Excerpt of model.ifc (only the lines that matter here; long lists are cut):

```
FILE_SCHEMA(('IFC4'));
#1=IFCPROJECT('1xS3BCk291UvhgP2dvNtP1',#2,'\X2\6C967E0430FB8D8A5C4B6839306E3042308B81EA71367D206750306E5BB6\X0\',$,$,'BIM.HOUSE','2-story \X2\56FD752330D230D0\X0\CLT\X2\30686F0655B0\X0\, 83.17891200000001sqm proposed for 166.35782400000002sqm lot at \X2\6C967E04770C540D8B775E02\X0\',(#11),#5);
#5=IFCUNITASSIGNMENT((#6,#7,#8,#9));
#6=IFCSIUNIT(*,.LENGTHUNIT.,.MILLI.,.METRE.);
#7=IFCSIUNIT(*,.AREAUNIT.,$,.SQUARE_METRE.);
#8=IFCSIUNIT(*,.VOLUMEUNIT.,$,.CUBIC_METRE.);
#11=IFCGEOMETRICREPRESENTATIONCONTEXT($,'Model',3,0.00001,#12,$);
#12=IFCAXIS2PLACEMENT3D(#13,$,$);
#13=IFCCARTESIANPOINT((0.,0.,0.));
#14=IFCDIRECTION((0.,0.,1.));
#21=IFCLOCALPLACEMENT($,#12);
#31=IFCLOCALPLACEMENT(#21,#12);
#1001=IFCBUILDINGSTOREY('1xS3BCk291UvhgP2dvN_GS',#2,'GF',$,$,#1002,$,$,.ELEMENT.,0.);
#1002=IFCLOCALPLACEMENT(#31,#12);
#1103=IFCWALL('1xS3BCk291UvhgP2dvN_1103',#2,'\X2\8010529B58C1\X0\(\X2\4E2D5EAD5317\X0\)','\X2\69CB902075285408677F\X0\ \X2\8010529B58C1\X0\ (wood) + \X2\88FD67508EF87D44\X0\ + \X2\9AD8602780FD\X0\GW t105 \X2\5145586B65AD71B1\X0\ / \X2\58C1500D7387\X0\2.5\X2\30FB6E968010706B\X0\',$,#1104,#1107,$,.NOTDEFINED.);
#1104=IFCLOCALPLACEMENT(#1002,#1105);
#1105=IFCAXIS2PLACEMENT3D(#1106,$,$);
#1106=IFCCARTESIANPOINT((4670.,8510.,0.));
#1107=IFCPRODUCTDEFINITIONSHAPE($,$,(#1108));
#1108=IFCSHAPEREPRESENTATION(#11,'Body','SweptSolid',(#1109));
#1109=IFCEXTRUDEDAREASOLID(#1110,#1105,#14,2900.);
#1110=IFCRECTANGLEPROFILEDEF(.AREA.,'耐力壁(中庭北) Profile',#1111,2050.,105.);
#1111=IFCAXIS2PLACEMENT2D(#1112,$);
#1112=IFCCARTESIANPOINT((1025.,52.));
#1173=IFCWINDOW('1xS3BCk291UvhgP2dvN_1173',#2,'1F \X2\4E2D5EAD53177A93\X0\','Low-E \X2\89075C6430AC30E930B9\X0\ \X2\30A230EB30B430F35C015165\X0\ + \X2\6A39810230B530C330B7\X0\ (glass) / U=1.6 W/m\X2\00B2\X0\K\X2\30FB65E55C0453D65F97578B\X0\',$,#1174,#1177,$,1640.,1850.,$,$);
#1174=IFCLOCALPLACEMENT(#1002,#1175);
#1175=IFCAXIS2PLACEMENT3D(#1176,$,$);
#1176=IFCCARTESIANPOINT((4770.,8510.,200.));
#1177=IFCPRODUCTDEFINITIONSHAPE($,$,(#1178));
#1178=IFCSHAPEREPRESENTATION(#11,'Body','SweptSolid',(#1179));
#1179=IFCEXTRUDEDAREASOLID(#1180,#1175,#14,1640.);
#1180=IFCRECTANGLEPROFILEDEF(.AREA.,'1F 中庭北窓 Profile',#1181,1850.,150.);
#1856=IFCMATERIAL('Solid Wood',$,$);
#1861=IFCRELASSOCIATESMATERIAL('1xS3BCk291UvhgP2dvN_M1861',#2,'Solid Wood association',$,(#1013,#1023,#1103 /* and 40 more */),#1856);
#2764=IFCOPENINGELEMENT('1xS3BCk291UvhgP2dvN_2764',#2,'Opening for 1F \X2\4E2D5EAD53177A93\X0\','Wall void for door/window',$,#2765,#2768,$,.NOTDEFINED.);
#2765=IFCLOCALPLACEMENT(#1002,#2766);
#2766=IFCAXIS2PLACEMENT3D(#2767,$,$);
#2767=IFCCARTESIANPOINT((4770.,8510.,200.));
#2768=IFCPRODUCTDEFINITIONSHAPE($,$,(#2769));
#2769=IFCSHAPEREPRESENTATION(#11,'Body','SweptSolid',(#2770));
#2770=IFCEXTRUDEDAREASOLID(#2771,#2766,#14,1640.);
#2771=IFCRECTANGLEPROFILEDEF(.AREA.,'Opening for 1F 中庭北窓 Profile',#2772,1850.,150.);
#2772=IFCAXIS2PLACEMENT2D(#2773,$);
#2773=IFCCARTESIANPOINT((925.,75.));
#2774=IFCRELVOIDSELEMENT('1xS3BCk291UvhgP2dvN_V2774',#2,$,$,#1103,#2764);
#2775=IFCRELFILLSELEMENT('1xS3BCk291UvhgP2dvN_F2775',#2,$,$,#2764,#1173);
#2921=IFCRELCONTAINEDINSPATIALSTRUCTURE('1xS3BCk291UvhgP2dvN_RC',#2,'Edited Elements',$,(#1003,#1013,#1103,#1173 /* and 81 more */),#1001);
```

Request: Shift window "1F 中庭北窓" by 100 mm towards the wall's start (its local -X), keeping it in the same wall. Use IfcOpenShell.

```python
import ifcopenshell
import ifcopenshell.api.geometry
import ifcopenshell.util.placement

model = ifcopenshell.open("model.ifc")

window = model.by_guid("1xS3BCk291UvhgP2dvN_1173")
opening = window.FillsVoids[0].RelatingOpeningElement
wall = opening.VoidsElements[0].RelatingBuildingElement

wall_matrix = ifcopenshell.util.placement.get_local_placement(wall.ObjectPlacement)
shift = wall_matrix[:3, 0] * -100.0
before = ifcopenshell.util.placement.get_local_placement(window.ObjectPlacement)[:3, 3].copy()

# The window is not placed relative to its opening, so move both.
for product in (opening, window):
    matrix = ifcopenshell.util.placement.get_local_placement(product.ObjectPlacement)
    matrix[:3, 3] += shift
    ifcopenshell.api.geometry.edit_object_placement(model, product=product, matrix=matrix, is_si=False)

after = ifcopenshell.util.placement.get_local_placement(window.ObjectPlacement)[:3, 3]
print("window moved by", (after - before).round(3) + 0.0)

model.write("model_rev.ifc")
```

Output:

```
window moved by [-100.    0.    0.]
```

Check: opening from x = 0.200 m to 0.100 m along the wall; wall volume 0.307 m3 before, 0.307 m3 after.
